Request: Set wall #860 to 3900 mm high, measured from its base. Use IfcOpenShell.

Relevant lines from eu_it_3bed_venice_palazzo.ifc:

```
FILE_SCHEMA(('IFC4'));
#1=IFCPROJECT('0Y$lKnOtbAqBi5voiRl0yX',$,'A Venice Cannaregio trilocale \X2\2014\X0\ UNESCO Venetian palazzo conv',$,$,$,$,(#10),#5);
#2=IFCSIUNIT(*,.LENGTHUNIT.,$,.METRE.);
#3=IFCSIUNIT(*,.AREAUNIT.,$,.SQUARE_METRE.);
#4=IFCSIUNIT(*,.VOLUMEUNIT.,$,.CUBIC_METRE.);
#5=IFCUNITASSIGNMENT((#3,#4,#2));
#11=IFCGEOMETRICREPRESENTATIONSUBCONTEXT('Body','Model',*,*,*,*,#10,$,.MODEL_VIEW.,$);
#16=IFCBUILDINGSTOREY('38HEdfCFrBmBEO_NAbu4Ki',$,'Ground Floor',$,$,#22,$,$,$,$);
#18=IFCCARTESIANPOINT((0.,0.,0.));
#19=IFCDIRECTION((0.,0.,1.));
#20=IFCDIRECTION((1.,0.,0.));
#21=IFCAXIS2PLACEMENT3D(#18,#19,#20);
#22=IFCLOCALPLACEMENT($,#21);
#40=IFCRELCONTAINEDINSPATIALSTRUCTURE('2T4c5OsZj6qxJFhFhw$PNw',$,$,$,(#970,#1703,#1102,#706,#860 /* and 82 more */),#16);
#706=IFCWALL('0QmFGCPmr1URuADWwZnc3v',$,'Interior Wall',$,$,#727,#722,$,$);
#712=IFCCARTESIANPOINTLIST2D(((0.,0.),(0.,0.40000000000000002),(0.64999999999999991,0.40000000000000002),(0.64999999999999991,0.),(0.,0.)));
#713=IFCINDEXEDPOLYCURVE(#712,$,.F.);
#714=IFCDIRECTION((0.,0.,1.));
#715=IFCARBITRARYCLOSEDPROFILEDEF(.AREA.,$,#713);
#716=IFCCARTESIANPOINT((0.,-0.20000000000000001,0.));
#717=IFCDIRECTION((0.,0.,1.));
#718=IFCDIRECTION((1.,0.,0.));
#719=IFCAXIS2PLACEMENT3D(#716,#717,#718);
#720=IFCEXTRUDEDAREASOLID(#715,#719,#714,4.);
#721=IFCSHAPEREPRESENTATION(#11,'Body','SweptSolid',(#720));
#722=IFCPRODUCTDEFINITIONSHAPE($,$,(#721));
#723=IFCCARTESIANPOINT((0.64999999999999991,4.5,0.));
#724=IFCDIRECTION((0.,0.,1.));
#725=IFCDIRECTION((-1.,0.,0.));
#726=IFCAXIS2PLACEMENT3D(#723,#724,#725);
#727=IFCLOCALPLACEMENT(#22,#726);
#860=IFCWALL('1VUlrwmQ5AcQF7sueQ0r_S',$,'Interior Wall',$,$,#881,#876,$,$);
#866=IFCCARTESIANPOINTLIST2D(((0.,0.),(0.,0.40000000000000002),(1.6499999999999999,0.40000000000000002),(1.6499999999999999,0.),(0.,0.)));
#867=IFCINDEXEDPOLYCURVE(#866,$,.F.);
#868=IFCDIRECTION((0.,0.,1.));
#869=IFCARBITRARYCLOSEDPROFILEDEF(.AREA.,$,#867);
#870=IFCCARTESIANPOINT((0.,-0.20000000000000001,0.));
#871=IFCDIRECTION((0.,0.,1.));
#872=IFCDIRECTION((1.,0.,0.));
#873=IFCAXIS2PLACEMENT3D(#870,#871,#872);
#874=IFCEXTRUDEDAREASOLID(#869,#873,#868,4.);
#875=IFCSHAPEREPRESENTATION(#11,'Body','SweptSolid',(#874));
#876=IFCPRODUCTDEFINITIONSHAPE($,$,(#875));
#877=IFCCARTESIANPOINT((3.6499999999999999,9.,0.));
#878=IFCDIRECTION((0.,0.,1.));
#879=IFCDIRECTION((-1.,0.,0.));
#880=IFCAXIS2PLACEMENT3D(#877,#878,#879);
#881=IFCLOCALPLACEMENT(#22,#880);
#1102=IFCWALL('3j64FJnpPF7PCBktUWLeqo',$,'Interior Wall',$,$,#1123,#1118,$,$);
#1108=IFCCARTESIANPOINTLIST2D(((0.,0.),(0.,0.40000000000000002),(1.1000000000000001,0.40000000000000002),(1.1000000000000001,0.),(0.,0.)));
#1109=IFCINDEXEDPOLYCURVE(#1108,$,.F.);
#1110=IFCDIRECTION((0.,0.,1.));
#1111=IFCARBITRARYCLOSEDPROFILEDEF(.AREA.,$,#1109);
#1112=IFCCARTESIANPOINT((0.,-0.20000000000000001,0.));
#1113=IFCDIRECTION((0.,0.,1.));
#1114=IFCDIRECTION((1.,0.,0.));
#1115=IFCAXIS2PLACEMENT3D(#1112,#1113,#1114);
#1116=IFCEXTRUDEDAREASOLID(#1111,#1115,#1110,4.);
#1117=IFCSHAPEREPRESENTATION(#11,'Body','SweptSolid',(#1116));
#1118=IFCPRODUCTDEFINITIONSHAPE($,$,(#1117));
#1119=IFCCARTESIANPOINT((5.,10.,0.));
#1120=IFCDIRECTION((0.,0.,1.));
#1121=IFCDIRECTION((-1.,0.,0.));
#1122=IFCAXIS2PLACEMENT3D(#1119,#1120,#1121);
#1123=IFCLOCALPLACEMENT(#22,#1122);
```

```python
import ifcopenshell
import ifcopenshell.geom
import ifcopenshell.util.representation
import ifcopenshell.util.shape

model = ifcopenshell.open("eu_it_3bed_venice_palazzo.ifc")
settings = ifcopenshell.geom.settings()


def volume(element):
    """Net volume in cubic metres, openings subtracted."""
    shape = ifcopenshell.geom.create_shape(settings, element)
    return ifcopenshell.util.shape.get_volume(shape.geometry)


wall = model.by_id(860)
before = volume(wall)

body = ifcopenshell.util.representation.get_representation(wall, "Model", "Body")
solid = body.Items[0]
old_height = solid.Depth
solid.Depth = 3.9
after = volume(wall)

print(f"height {old_height:g} -> {solid.Depth:g}, volume {before:.3f} -> {after:.3f} m3")

model.write("eu_it_3bed_venice_palazzo_rev.ifc")
```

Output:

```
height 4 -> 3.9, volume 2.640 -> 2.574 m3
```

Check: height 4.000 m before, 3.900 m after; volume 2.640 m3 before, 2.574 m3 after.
